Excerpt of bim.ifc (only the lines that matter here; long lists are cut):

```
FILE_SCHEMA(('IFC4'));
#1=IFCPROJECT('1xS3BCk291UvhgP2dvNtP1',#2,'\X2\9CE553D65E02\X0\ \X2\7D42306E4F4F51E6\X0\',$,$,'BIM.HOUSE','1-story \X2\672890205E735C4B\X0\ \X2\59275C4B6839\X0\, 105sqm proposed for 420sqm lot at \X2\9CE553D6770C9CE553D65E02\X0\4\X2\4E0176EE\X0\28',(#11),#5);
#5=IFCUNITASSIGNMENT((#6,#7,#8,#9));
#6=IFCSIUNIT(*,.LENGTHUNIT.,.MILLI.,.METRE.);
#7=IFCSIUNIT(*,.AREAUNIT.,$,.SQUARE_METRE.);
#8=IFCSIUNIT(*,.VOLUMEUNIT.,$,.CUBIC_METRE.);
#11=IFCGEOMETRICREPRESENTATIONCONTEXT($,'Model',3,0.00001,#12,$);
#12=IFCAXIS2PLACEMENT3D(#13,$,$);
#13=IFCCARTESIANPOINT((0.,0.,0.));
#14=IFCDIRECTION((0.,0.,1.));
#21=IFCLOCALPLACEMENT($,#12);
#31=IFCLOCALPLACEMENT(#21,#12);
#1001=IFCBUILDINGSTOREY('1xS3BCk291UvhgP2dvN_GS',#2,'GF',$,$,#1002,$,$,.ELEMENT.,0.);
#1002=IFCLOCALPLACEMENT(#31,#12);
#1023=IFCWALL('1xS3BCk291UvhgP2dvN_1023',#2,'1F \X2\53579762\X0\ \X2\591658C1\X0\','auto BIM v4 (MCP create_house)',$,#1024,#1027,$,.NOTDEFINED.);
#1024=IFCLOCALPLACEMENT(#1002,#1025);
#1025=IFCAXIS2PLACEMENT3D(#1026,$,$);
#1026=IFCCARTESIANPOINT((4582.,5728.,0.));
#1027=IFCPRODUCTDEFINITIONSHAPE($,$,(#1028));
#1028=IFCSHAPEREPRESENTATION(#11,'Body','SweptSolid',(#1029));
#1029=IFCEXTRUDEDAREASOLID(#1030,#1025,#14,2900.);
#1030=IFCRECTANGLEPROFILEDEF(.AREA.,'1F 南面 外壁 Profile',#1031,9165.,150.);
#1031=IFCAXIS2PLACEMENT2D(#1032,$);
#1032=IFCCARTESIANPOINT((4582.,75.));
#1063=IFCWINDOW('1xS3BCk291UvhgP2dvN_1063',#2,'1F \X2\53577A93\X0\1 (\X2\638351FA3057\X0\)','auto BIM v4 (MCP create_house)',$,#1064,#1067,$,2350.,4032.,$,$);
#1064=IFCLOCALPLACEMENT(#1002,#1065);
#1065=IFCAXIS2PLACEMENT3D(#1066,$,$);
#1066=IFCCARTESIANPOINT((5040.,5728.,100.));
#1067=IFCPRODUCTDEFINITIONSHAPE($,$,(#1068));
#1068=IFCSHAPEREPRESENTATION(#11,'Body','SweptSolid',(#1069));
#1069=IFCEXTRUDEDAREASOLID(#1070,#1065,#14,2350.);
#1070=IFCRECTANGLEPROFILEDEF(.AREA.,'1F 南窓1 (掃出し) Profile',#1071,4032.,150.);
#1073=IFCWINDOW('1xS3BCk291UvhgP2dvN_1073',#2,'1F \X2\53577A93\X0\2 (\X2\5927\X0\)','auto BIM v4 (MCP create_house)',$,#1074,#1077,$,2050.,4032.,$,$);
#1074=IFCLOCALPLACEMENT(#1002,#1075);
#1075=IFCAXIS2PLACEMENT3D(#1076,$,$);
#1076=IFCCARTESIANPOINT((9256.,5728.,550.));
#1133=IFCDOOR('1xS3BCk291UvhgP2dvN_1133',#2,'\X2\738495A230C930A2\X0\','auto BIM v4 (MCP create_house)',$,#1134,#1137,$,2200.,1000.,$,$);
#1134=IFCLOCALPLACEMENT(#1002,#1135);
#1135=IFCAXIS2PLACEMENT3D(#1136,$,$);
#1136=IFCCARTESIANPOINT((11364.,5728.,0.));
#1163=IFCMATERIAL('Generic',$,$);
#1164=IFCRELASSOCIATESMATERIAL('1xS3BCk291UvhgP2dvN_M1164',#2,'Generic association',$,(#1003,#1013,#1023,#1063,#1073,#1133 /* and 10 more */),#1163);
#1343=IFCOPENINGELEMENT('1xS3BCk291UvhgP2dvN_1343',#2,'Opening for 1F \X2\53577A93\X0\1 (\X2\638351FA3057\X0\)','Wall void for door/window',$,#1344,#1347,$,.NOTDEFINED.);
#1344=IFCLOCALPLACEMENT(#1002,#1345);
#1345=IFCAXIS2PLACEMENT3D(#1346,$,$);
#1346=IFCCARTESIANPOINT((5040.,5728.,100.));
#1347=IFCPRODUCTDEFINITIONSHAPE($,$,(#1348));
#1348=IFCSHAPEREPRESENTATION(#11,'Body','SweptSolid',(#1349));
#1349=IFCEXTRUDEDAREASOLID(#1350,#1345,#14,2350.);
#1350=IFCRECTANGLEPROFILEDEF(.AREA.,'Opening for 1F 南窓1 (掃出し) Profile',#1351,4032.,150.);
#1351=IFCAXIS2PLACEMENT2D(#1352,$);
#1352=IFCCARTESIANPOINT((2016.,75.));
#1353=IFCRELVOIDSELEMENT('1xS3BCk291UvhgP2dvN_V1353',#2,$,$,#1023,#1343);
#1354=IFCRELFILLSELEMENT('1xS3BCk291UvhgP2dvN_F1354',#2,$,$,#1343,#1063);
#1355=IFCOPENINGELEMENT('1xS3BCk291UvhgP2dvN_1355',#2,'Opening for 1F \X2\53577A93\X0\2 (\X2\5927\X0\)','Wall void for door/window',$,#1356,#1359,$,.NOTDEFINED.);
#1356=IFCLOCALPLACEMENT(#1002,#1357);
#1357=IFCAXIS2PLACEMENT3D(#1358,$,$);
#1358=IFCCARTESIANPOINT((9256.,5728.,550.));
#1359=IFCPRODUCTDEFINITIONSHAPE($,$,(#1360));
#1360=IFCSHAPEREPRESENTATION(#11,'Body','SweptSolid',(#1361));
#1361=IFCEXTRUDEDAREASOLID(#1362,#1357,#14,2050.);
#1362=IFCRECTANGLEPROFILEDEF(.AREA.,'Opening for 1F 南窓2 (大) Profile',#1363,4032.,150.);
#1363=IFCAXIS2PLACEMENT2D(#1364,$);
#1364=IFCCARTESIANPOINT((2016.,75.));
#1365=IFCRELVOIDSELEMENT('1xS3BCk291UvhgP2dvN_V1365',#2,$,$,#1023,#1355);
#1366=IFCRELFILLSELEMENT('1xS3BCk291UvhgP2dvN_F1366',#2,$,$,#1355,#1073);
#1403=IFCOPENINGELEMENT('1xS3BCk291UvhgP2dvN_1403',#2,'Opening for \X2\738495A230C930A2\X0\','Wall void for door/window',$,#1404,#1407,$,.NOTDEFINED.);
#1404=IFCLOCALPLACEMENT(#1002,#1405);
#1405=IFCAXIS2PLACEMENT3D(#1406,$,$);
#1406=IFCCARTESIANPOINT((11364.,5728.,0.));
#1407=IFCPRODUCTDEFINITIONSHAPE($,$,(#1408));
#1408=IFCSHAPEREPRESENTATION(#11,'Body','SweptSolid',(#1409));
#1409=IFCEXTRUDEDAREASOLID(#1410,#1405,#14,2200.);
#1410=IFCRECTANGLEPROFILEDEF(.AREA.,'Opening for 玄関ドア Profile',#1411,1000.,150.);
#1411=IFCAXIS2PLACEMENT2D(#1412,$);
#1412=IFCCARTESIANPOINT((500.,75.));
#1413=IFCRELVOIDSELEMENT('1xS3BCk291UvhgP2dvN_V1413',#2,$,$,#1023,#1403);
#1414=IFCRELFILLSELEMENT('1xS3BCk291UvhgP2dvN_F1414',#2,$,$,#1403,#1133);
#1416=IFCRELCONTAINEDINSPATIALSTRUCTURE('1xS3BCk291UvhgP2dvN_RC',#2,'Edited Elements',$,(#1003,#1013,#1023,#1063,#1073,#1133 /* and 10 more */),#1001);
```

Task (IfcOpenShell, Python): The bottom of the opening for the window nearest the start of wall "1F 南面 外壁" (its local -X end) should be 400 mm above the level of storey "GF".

```python
import numpy as np
import ifcopenshell
import ifcopenshell.api.geometry
import ifcopenshell.geom
import ifcopenshell.util.element
import ifcopenshell.util.placement
import ifcopenshell.util.shape
import ifcopenshell.util.unit

model = ifcopenshell.open("bim.ifc")
unit_scale = ifcopenshell.util.unit.calculate_unit_scale(model)

window = model.by_id(1063)
opening = window.FillsVoids[0].RelatingOpeningElement
storey = ifcopenshell.util.element.get_container(window, ifc_class="IfcBuildingStorey")
level = ifcopenshell.util.placement.get_local_placement(storey.ObjectPlacement)[2, 3]

# The opening's origin need not be at the sill, so measure its lowest point.
shape = ifcopenshell.geom.create_shape(ifcopenshell.geom.settings(), opening)
bottom = ifcopenshell.util.shape.get_shape_bottom_elevation(shape, shape.geometry) / unit_scale
dz = level + 400.0 - bottom

shift = np.array([0.0, 0.0, dz])
# The window is not placed relative to its opening, so move both.
for product in (opening, window):
    matrix = ifcopenshell.util.placement.get_local_placement(product.ObjectPlacement)
    matrix[:3, 3] += shift
    ifcopenshell.api.geometry.edit_object_placement(model, product=product, matrix=matrix, is_si=False)

print(f"moved by {dz * unit_scale:+.3f} m")

model.write("bim_rev.ifc")
```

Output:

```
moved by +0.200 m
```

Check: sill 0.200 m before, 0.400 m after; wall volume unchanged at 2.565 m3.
